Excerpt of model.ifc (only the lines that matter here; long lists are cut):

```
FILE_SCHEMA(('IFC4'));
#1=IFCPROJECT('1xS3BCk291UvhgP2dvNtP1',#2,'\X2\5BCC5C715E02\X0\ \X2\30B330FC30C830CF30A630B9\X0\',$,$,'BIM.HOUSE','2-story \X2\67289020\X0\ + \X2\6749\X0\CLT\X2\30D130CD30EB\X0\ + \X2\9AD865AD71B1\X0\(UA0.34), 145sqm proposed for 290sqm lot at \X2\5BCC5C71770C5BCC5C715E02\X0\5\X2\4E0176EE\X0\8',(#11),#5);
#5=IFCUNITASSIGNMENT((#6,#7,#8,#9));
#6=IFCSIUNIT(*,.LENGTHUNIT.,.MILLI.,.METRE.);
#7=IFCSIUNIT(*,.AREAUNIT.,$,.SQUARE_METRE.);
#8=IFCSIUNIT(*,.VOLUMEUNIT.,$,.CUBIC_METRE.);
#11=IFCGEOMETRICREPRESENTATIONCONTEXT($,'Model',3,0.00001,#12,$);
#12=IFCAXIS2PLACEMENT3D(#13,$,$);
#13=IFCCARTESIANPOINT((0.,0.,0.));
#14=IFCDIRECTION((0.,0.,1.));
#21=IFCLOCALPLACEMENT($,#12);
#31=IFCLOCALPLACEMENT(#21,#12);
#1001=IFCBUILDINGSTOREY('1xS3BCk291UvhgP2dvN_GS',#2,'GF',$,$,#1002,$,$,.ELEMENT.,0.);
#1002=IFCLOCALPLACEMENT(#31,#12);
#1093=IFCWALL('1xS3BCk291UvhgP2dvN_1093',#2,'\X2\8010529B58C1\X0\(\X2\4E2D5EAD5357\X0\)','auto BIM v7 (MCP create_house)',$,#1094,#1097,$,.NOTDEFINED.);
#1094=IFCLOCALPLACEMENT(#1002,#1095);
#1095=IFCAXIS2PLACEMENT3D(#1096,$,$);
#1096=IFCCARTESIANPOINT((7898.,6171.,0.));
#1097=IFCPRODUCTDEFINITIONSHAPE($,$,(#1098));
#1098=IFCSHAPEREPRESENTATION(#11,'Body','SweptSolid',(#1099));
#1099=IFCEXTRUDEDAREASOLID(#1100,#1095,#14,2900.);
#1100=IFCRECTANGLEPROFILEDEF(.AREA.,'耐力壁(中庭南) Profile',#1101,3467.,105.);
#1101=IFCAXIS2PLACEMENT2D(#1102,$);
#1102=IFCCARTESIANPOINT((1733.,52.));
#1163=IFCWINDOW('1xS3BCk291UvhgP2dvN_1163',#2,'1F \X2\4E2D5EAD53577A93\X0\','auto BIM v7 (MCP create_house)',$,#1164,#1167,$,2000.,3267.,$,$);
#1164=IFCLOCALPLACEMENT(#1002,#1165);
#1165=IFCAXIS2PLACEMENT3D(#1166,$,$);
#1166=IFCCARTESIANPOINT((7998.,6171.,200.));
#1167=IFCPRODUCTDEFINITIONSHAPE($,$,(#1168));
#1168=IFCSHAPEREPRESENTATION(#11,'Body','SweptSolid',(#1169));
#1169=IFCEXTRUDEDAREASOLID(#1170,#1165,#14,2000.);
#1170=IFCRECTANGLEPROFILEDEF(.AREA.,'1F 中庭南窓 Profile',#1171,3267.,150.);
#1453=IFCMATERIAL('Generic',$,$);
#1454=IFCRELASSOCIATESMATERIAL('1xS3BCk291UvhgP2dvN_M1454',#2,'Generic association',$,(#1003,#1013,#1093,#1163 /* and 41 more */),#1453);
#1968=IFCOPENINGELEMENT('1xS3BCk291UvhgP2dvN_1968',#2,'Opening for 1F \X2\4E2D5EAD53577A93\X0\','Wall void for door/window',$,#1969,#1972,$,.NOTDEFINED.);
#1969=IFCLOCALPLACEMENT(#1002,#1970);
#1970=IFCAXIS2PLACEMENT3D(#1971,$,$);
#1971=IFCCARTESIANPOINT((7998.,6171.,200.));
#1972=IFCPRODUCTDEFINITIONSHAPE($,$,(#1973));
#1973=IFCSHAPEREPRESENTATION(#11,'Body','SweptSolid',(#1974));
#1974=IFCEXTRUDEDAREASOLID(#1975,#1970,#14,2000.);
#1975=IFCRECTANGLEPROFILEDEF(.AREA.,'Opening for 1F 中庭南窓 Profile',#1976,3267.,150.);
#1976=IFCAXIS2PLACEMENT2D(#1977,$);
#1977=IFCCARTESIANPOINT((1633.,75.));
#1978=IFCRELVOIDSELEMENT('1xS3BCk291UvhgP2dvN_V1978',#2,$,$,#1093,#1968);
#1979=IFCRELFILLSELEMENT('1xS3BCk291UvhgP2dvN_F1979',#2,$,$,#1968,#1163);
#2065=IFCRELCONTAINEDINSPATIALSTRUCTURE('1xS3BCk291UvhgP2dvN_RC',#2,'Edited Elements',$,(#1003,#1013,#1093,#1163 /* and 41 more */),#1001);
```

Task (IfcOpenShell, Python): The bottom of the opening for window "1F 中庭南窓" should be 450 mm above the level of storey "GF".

```python
import numpy as np
import ifcopenshell
import ifcopenshell.api.geometry
import ifcopenshell.geom
import ifcopenshell.util.element
import ifcopenshell.util.placement
import ifcopenshell.util.shape
import ifcopenshell.util.unit

model = ifcopenshell.open("model.ifc")
unit_scale = ifcopenshell.util.unit.calculate_unit_scale(model)

window = model.by_guid("1xS3BCk291UvhgP2dvN_1163")
opening = window.FillsVoids[0].RelatingOpeningElement
storey = ifcopenshell.util.element.get_container(window, ifc_class="IfcBuildingStorey")
level = ifcopenshell.util.placement.get_local_placement(storey.ObjectPlacement)[2, 3]

# The opening's origin need not be at the sill, so measure its lowest point.
shape = ifcopenshell.geom.create_shape(ifcopenshell.geom.settings(), opening)
bottom = ifcopenshell.util.shape.get_shape_bottom_elevation(shape, shape.geometry) / unit_scale
dz = level + 450.0 - bottom

shift = np.array([0.0, 0.0, dz])
# The window is not placed relative to its opening, so move both.
for product in (opening, window):
    matrix = ifcopenshell.util.placement.get_local_placement(product.ObjectPlacement)
    matrix[:3, 3] += shift
    ifcopenshell.api.geometry.edit_object_placement(model, product=product, matrix=matrix, is_si=False)

print(f"moved by {dz * unit_scale:+.3f} m")

model.write("model_edited.ifc")
```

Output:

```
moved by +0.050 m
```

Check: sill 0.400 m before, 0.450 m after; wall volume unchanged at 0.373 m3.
